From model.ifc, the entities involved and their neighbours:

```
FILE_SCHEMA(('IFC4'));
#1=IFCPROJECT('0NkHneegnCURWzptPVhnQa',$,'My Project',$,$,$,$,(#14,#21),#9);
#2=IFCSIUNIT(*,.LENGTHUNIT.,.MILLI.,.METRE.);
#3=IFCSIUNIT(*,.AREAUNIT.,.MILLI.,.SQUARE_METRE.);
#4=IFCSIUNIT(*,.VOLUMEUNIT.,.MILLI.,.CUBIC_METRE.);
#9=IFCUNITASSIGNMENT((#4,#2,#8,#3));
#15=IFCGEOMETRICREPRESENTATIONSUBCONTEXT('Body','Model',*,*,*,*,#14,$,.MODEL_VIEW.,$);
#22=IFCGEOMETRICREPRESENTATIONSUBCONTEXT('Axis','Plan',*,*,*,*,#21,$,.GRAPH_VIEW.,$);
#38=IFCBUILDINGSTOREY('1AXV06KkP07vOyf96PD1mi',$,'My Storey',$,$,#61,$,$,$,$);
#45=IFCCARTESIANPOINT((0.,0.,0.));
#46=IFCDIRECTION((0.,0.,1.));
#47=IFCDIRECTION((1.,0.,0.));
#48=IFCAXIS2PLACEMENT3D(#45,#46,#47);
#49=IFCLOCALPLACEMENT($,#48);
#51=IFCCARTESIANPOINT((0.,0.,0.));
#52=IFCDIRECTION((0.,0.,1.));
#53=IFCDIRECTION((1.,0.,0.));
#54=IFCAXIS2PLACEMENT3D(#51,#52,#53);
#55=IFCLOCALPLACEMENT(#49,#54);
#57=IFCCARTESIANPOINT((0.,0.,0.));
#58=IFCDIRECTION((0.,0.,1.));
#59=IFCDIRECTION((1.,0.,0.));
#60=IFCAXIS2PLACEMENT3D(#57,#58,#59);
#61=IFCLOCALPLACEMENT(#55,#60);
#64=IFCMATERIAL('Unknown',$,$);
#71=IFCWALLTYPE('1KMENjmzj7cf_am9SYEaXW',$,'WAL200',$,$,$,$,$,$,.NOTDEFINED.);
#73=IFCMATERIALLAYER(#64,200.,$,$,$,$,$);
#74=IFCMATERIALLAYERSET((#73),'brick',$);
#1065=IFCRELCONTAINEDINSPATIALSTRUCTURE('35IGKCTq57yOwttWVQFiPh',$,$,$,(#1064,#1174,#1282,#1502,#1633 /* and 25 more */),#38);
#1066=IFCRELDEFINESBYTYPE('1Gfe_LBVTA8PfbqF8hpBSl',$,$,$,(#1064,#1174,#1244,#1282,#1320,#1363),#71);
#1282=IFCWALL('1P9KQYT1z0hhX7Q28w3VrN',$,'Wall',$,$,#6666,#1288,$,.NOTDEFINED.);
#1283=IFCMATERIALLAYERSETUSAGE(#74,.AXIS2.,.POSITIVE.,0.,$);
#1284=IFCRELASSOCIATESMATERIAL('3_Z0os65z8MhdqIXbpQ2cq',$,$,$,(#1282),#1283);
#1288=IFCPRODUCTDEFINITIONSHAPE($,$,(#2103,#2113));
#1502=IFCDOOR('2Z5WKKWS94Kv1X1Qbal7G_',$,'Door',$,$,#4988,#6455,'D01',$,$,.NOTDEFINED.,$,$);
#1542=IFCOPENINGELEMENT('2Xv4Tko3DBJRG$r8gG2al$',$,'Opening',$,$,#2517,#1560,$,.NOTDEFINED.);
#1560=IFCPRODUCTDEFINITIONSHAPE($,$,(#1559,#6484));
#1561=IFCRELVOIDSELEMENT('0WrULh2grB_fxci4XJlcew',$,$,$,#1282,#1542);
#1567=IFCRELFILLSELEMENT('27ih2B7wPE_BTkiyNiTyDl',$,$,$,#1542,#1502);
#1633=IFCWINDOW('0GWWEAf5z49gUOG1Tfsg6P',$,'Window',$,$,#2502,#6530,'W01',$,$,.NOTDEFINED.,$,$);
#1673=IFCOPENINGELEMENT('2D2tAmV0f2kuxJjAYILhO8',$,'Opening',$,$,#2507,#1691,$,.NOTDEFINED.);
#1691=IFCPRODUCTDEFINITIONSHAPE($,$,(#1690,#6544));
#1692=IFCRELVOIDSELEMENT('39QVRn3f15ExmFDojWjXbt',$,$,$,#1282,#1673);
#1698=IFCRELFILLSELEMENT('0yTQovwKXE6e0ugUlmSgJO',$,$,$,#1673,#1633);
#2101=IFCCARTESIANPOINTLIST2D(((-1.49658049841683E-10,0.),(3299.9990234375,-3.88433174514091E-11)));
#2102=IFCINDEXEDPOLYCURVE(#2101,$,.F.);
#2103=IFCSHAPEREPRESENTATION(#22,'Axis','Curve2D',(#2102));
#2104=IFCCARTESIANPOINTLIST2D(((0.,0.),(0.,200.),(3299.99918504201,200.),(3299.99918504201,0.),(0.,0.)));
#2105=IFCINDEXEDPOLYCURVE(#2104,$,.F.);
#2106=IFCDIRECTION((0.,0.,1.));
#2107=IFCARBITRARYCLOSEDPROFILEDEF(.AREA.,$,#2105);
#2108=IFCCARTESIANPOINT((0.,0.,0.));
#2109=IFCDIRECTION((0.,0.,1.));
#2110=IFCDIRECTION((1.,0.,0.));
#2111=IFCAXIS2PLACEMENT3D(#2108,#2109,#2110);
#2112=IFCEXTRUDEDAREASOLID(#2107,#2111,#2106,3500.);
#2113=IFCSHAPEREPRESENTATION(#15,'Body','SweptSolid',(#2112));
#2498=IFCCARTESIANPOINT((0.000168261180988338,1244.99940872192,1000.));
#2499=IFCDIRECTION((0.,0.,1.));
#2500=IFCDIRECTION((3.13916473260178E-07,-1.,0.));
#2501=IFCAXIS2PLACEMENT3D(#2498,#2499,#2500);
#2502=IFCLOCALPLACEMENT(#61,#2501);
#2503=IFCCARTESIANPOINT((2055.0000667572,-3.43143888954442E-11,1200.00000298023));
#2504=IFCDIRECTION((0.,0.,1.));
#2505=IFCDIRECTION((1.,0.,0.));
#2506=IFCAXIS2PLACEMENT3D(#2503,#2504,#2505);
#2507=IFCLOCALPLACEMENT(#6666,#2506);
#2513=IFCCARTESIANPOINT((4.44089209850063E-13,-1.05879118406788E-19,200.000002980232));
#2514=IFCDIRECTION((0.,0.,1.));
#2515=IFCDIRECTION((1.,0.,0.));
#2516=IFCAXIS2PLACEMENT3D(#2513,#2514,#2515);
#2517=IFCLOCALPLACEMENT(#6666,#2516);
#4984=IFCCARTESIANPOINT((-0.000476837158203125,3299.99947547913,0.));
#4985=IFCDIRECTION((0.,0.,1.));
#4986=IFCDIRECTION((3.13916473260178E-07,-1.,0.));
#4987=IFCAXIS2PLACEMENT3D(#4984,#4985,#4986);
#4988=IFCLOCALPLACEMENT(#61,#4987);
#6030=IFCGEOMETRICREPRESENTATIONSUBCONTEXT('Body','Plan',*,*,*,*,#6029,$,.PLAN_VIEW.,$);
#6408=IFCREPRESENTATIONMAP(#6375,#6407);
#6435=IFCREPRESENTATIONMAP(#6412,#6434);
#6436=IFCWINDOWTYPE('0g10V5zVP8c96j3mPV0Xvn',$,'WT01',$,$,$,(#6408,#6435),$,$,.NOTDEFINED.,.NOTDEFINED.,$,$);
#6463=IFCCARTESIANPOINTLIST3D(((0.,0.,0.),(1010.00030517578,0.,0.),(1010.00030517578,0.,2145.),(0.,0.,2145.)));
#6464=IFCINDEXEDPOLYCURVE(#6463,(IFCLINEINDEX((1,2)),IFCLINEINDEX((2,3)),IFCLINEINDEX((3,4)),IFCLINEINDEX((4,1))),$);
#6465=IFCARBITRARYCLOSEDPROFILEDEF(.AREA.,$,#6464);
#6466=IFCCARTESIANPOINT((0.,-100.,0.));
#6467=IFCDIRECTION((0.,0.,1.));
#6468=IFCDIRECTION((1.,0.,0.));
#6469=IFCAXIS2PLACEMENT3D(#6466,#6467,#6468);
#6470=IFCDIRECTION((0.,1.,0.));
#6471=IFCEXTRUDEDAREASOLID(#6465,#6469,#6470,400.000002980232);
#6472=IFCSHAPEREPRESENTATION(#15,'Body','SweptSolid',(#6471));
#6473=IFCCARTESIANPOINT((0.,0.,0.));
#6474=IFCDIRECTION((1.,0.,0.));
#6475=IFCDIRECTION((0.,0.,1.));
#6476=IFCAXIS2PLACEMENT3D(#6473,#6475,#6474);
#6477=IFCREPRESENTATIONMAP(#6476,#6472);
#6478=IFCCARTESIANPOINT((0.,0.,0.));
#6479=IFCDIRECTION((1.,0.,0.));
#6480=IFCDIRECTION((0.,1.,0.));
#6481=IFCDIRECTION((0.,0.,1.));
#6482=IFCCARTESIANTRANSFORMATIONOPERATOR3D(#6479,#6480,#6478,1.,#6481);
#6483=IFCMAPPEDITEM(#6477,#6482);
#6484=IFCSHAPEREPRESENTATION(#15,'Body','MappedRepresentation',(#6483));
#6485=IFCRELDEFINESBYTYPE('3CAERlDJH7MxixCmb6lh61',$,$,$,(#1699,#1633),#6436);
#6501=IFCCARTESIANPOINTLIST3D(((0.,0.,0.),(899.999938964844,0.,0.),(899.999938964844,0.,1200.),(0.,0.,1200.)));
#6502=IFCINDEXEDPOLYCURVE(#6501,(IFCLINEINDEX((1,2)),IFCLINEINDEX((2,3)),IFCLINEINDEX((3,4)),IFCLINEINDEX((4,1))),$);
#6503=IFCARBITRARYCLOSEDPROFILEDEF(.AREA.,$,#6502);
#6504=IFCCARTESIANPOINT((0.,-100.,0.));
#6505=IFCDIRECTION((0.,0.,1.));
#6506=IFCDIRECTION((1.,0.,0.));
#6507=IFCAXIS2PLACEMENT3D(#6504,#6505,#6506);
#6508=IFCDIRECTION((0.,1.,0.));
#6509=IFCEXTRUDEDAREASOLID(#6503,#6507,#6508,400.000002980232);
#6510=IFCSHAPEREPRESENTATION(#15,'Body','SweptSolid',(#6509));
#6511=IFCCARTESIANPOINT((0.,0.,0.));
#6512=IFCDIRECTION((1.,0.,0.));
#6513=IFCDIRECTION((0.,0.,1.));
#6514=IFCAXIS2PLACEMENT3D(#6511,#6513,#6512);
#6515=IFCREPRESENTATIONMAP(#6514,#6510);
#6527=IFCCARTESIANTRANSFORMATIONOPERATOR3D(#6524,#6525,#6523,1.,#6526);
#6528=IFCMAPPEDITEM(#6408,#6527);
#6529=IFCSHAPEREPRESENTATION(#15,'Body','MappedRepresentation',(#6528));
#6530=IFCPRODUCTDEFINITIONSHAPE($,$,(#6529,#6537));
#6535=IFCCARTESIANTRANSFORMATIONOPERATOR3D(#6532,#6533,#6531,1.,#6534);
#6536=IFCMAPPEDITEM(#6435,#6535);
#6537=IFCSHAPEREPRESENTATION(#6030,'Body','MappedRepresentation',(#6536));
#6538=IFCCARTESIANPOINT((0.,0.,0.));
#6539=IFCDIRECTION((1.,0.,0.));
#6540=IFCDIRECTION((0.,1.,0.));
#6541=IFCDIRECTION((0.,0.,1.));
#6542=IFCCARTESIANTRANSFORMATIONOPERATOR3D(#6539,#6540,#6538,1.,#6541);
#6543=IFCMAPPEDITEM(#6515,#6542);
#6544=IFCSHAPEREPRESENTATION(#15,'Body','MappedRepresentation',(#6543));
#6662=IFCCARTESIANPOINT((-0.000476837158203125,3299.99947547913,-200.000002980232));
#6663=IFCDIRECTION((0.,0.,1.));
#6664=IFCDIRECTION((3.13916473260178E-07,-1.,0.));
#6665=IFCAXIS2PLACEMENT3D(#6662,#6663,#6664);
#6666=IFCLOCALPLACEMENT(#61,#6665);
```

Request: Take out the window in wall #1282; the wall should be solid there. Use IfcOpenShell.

```python
import ifcopenshell
import ifcopenshell.api.feature
import ifcopenshell.api.root
import ifcopenshell.geom
import ifcopenshell.util.shape

model = ifcopenshell.open("model.ifc")
settings = ifcopenshell.geom.settings()


def volume(element):
    """Net volume in cubic metres, openings subtracted."""
    shape = ifcopenshell.geom.create_shape(settings, element)
    return ifcopenshell.util.shape.get_volume(shape.geometry)


window = model.by_guid("0GWWEAf5z49gUOG1Tfsg6P")
opening = window.FillsVoids[0].RelatingOpeningElement
wall = opening.VoidsElements[0].RelatingBuildingElement
before = volume(wall)

ifcopenshell.api.root.remove_product(model, product=window)
ifcopenshell.api.feature.remove_feature(model, feature=opening)

after = volume(wall)

print(f"wall volume {before:.3f} -> {after:.3f} m3")

model.write("model_v2.ifc")
```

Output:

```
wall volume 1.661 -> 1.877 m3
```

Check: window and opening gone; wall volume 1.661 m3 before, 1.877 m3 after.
